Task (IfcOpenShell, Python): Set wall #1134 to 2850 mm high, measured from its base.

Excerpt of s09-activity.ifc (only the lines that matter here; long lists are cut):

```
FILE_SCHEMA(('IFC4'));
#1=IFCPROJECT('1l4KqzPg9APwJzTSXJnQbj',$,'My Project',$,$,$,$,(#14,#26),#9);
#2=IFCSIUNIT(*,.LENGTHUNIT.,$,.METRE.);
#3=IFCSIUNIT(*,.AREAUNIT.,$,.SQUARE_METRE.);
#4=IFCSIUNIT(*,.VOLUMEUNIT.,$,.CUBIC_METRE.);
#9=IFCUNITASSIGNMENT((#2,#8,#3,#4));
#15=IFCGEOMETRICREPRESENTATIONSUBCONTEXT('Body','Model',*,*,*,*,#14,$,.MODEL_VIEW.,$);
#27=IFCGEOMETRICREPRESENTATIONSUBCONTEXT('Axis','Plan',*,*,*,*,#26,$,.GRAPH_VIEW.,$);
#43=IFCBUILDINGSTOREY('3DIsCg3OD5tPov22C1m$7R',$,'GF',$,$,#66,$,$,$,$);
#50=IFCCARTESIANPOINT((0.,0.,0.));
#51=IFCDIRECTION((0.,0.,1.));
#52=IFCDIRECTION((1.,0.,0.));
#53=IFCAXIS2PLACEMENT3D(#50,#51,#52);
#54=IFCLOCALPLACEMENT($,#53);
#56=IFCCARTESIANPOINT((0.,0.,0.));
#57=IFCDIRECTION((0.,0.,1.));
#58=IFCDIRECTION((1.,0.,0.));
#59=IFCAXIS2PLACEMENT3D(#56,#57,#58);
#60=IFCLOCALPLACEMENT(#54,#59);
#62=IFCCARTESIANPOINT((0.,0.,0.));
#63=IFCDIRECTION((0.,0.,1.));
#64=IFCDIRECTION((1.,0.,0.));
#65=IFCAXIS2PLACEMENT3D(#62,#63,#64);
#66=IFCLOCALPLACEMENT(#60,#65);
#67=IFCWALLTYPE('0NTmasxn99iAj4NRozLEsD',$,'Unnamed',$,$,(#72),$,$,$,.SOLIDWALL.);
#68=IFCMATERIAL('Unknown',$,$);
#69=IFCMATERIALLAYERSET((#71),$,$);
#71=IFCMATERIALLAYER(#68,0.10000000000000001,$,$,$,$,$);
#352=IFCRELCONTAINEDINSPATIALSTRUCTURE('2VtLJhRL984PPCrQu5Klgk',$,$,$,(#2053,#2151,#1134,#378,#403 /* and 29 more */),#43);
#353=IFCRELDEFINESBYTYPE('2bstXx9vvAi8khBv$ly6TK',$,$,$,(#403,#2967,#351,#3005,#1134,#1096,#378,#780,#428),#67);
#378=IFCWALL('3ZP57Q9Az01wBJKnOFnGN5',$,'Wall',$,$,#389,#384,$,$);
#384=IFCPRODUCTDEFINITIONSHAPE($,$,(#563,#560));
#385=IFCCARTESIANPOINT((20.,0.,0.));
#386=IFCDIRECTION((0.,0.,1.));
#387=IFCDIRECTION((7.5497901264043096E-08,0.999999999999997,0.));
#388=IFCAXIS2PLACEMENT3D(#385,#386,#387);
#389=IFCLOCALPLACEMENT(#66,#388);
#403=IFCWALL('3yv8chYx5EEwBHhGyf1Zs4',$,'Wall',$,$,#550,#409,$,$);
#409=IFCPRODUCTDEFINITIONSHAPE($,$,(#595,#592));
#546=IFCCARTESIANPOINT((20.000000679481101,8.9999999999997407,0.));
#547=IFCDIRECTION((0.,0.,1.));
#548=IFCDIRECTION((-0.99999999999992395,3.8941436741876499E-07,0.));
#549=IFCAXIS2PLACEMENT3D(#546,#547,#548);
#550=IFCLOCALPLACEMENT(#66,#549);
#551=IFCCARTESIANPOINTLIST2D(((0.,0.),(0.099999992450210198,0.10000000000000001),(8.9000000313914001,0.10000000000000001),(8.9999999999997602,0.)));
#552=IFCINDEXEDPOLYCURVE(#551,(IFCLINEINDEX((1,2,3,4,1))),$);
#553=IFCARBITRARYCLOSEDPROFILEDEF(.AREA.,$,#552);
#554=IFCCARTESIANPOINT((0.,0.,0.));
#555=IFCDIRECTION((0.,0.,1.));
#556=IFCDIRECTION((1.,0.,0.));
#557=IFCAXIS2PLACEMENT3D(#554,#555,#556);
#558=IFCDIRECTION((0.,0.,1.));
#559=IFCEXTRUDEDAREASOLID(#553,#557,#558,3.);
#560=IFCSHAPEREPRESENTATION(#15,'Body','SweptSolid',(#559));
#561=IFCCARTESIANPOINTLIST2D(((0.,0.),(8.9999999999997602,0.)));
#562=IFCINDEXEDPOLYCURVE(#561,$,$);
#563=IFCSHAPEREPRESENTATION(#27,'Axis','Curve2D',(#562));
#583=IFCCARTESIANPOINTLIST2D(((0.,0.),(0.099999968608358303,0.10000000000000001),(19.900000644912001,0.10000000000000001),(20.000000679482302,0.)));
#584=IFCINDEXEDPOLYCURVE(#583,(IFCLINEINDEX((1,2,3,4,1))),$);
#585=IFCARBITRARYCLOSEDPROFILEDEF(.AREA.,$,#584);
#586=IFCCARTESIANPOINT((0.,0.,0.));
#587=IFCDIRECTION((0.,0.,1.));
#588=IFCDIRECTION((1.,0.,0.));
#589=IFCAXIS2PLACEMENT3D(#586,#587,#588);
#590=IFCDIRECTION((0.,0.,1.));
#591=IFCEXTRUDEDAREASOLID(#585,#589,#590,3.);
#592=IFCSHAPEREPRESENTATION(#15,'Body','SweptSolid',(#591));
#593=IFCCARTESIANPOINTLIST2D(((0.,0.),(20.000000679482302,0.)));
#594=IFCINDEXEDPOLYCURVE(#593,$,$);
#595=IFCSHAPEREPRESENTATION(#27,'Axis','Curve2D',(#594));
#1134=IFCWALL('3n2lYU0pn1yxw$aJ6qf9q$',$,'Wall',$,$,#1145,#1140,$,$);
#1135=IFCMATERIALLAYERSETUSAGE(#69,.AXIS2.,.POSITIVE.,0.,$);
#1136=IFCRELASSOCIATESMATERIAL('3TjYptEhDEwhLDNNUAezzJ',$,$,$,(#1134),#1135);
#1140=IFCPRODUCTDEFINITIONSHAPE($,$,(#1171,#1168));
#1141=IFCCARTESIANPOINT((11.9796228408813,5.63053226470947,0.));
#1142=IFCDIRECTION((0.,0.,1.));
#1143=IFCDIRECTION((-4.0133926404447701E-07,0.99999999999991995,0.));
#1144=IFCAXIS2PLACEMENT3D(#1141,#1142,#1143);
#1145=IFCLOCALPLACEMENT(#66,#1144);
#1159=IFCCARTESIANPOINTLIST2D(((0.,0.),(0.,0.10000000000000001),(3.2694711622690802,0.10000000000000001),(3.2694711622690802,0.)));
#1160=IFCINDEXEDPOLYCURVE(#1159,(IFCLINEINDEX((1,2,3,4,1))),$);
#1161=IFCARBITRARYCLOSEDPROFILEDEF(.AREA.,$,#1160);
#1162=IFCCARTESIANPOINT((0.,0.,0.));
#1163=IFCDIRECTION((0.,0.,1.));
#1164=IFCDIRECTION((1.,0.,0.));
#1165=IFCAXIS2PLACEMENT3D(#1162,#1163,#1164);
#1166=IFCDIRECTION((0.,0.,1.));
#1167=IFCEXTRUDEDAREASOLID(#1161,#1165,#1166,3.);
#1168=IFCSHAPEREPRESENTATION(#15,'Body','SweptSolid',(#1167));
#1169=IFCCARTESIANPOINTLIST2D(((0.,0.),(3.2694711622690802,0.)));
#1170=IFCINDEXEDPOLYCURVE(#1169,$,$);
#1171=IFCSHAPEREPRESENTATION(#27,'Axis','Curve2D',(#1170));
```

```python
import ifcopenshell
import ifcopenshell.geom
import ifcopenshell.util.representation
import ifcopenshell.util.shape
import ifcopenshell.util.unit

model = ifcopenshell.open("s09-activity.ifc")
unit_scale = ifcopenshell.util.unit.calculate_unit_scale(model)
settings = ifcopenshell.geom.settings()


def volume(element):
    """Net volume in cubic metres, openings subtracted."""
    shape = ifcopenshell.geom.create_shape(settings, element)
    return ifcopenshell.util.shape.get_volume(shape.geometry)


wall = model.by_guid("3n2lYU0pn1yxw$aJ6qf9q$")
before = volume(wall)

body = ifcopenshell.util.representation.get_representation(wall, "Model", "Body")
solid = body.Items[0]
old_height = solid.Depth
solid.Depth = 2.85 / unit_scale
after = volume(wall)

print(f"height {old_height:g} -> {solid.Depth:g}, volume {before:.3f} -> {after:.3f} m3")

model.write("s09-activity-out.ifc")
```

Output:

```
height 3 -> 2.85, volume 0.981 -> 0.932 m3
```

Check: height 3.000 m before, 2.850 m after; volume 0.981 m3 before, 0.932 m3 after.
